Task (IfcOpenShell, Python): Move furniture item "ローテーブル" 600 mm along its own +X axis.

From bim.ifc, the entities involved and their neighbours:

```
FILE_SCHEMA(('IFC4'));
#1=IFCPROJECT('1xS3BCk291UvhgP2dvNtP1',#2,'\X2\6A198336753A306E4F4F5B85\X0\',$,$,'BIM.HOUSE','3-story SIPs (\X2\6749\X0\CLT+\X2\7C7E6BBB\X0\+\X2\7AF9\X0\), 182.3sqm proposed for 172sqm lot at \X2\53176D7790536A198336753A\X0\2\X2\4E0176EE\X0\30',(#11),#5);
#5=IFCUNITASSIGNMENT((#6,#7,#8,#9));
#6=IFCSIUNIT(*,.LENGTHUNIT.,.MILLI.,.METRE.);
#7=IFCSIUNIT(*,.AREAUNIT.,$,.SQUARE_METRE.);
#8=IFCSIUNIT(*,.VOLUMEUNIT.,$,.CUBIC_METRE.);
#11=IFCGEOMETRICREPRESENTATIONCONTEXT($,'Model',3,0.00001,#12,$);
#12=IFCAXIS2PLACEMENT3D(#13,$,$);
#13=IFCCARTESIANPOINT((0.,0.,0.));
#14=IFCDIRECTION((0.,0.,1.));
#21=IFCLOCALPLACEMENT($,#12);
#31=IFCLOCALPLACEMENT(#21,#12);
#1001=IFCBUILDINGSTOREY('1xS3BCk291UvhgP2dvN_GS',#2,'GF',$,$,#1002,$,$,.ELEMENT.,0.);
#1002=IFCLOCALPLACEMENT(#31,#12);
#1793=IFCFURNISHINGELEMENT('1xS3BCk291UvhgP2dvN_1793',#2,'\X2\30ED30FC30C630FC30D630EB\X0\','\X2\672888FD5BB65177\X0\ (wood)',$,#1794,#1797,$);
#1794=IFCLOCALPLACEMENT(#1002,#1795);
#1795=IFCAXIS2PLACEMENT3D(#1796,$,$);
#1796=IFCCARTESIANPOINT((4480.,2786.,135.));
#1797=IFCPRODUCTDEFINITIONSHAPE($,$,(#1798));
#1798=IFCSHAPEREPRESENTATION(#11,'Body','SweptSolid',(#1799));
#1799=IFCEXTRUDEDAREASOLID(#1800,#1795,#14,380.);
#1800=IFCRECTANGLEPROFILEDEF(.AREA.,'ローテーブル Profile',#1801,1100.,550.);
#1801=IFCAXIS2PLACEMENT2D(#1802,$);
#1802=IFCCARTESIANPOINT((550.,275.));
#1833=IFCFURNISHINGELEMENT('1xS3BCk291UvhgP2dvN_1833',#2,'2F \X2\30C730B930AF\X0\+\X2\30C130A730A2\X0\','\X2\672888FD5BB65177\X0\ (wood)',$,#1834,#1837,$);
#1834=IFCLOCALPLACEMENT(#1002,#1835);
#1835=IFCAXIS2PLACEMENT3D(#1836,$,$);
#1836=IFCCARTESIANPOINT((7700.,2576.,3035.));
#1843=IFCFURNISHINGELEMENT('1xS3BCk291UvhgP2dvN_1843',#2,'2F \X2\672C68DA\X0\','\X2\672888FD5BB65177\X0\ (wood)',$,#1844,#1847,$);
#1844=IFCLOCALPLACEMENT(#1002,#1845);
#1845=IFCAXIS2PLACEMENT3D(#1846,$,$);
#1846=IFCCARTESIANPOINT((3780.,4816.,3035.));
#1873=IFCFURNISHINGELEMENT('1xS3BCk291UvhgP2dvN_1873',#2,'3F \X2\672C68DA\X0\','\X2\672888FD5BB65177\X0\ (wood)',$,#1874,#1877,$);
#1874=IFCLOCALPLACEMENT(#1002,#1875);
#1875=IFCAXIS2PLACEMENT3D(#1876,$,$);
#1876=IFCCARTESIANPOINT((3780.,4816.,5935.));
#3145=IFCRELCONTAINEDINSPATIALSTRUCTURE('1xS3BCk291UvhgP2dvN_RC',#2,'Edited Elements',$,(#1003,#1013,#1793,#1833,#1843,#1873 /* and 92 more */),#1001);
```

```python
import ifcopenshell
import ifcopenshell.api.geometry
import ifcopenshell.util.placement
import ifcopenshell.util.unit

model = ifcopenshell.open("bim.ifc")
unit_scale = ifcopenshell.util.unit.calculate_unit_scale(model)

item = model.by_guid("1xS3BCk291UvhgP2dvN_1793")
matrix = ifcopenshell.util.placement.get_local_placement(item.ObjectPlacement)
matrix[:3, 3] += matrix[:3, 0] * 0.6 / unit_scale
ifcopenshell.api.geometry.edit_object_placement(model, product=item, matrix=matrix, is_si=False)

print(ifcopenshell.util.placement.get_local_placement(item.ObjectPlacement).round(3) + 0.0)

model.write("bim-out.ifc")
```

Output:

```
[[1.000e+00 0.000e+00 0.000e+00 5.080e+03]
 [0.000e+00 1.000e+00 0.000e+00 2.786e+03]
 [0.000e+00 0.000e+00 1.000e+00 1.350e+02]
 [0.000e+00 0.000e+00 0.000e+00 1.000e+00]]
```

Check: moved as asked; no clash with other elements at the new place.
